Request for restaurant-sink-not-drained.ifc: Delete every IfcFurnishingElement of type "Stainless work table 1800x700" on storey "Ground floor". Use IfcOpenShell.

First a look at what the model holds.

```python
import ifcopenshell
import ifcopenshell.util.element

model = ifcopenshell.open("restaurant-sink-not-drained.ifc")
print(model.schema)
storey = next(s for s in model.by_type("IfcBuildingStorey") if s.Name == "Ground floor")
furniture = [e for e in ifcopenshell.util.element.get_decomposition(storey) if e.is_a("IfcFurnishingElement")]
seen = {}
for e in furniture:
    element_type = ifcopenshell.util.element.get_type(e)
    name = element_type.Name if element_type not in (None, e) else None
    seen[name] = seen.get(name, 0) + 1
for name, count in sorted(seen.items(), key=str):
    print(count, "x", name)
```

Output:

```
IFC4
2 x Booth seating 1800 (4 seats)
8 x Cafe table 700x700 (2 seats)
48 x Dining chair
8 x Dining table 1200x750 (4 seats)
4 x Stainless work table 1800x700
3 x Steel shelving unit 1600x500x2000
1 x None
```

```python
import ifcopenshell
import ifcopenshell.api.root
import ifcopenshell.util.element

model = ifcopenshell.open("restaurant-sink-not-drained.ifc")

storey = next(s for s in model.by_type("IfcBuildingStorey") if s.Name == "Ground floor")
furniture = [e for e in ifcopenshell.util.element.get_decomposition(storey) if e.is_a("IfcFurnishingElement")]
targets = [e for e in furniture if (t := ifcopenshell.util.element.get_type(e)) not in (None, e) and t.Name == "Stainless work table 1800x700"]

for e in targets:
    ifcopenshell.api.root.remove_product(model, product=e)
print(len(targets), "removed")

model.write("restaurant-sink-not-drained_rev.ifc")
```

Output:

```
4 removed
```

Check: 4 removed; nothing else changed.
